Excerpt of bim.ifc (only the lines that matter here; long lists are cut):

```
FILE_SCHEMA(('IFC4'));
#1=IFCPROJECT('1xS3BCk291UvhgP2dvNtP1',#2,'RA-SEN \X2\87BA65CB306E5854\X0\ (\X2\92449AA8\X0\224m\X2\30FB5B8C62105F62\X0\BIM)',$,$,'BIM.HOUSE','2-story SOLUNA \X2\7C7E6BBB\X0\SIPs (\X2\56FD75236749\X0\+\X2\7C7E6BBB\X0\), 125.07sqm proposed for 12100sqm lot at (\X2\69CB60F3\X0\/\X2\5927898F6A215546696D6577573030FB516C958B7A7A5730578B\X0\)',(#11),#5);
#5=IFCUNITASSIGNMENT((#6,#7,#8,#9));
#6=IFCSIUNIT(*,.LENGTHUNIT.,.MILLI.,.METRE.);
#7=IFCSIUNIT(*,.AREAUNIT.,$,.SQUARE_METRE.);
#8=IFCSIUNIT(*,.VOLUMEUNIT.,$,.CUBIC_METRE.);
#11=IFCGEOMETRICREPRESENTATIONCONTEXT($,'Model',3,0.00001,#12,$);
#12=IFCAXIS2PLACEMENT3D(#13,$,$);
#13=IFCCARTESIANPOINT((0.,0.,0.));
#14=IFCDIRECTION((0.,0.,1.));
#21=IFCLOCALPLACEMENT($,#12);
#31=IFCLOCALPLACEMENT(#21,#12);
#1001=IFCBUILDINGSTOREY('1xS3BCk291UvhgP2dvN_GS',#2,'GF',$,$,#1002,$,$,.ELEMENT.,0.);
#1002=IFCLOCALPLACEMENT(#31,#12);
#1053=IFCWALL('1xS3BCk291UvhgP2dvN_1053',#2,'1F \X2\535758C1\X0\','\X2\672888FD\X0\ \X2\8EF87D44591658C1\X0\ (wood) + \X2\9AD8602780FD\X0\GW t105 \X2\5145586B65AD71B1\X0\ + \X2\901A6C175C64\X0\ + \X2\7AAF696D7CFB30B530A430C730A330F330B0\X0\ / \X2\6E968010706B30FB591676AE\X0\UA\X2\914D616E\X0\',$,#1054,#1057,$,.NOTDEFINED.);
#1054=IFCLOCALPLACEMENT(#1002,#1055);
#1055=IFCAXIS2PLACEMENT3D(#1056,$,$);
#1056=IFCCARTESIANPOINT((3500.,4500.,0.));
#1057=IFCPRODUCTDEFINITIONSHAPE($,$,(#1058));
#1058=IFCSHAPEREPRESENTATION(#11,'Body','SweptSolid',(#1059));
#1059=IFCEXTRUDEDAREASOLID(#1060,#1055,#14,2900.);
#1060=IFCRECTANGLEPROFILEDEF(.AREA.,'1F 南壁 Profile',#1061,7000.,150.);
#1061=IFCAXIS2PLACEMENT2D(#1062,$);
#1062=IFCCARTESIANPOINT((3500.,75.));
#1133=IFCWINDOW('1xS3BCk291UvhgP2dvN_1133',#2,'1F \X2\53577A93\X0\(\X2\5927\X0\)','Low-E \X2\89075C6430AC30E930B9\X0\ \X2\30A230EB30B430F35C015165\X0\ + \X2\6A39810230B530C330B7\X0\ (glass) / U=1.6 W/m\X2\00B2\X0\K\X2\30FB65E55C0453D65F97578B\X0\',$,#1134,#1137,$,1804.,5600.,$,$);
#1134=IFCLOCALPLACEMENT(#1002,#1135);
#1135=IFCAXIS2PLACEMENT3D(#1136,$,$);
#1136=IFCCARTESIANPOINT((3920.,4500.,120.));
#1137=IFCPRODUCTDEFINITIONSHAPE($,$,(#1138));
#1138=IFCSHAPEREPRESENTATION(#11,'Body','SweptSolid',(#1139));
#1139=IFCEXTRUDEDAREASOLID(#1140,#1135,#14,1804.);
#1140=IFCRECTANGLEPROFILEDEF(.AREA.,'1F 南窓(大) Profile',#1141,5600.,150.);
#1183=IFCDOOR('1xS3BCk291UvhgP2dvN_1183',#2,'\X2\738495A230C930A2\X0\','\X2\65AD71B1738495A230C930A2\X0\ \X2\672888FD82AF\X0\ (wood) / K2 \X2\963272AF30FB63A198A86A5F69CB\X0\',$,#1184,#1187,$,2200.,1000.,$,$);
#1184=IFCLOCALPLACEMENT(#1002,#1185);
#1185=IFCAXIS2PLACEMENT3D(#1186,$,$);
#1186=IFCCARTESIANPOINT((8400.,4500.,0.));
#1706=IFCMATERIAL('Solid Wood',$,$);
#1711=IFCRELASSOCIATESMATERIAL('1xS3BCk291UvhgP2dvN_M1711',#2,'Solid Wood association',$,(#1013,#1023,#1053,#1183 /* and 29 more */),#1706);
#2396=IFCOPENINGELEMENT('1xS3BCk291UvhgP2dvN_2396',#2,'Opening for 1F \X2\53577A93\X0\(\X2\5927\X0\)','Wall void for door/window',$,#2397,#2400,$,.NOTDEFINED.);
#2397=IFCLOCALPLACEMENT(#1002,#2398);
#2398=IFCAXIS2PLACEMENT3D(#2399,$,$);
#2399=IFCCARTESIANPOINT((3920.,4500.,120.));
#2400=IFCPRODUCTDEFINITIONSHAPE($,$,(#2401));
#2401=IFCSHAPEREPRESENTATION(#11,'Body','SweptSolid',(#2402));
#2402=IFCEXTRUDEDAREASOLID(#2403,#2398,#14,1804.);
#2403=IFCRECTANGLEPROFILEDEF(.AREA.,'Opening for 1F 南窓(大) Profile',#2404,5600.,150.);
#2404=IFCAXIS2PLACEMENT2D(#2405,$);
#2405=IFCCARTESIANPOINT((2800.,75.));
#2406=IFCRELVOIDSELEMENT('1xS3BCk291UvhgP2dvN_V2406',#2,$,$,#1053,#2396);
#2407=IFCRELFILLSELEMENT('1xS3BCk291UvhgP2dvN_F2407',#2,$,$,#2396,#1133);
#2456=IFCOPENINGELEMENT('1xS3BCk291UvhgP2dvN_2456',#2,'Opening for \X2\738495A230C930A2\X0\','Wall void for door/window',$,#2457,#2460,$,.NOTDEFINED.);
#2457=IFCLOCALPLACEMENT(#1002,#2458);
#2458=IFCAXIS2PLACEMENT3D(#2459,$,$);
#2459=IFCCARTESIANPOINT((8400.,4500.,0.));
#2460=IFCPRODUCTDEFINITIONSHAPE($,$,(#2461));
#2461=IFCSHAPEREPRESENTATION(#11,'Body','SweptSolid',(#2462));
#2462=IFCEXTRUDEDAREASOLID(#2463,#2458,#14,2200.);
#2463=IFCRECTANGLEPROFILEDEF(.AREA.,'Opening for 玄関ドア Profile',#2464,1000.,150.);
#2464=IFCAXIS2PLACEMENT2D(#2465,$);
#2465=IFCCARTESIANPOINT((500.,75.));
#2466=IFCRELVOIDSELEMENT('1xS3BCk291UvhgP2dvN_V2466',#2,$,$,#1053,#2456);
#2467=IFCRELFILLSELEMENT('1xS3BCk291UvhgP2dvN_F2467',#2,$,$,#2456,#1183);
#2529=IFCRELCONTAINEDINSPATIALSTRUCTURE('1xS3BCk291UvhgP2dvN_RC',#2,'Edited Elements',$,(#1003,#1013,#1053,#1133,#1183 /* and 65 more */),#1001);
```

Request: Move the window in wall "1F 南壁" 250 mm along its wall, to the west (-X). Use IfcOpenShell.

```python
import ifcopenshell
import ifcopenshell.api.geometry
import ifcopenshell.util.placement
import ifcopenshell.util.unit

model = ifcopenshell.open("bim.ifc")
unit_scale = ifcopenshell.util.unit.calculate_unit_scale(model)

window = model.by_guid("1xS3BCk291UvhgP2dvN_1133")
opening = window.FillsVoids[0].RelatingOpeningElement
wall = opening.VoidsElements[0].RelatingBuildingElement

wall_matrix = ifcopenshell.util.placement.get_local_placement(wall.ObjectPlacement)
shift = wall_matrix[:3, 0] * -0.25 / unit_scale
before = ifcopenshell.util.placement.get_local_placement(window.ObjectPlacement)[:3, 3].copy()

# The window is not placed relative to its opening, so move both.
for product in (opening, window):
    matrix = ifcopenshell.util.placement.get_local_placement(product.ObjectPlacement)
    matrix[:3, 3] += shift
    ifcopenshell.api.geometry.edit_object_placement(model, product=product, matrix=matrix, is_si=False)

after = ifcopenshell.util.placement.get_local_placement(window.ObjectPlacement)[:3, 3]
print("window moved by", (after - before).round(3) + 0.0)

model.write("bim_edited.ifc")
```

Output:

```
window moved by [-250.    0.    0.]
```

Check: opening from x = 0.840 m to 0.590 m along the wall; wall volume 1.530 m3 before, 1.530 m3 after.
